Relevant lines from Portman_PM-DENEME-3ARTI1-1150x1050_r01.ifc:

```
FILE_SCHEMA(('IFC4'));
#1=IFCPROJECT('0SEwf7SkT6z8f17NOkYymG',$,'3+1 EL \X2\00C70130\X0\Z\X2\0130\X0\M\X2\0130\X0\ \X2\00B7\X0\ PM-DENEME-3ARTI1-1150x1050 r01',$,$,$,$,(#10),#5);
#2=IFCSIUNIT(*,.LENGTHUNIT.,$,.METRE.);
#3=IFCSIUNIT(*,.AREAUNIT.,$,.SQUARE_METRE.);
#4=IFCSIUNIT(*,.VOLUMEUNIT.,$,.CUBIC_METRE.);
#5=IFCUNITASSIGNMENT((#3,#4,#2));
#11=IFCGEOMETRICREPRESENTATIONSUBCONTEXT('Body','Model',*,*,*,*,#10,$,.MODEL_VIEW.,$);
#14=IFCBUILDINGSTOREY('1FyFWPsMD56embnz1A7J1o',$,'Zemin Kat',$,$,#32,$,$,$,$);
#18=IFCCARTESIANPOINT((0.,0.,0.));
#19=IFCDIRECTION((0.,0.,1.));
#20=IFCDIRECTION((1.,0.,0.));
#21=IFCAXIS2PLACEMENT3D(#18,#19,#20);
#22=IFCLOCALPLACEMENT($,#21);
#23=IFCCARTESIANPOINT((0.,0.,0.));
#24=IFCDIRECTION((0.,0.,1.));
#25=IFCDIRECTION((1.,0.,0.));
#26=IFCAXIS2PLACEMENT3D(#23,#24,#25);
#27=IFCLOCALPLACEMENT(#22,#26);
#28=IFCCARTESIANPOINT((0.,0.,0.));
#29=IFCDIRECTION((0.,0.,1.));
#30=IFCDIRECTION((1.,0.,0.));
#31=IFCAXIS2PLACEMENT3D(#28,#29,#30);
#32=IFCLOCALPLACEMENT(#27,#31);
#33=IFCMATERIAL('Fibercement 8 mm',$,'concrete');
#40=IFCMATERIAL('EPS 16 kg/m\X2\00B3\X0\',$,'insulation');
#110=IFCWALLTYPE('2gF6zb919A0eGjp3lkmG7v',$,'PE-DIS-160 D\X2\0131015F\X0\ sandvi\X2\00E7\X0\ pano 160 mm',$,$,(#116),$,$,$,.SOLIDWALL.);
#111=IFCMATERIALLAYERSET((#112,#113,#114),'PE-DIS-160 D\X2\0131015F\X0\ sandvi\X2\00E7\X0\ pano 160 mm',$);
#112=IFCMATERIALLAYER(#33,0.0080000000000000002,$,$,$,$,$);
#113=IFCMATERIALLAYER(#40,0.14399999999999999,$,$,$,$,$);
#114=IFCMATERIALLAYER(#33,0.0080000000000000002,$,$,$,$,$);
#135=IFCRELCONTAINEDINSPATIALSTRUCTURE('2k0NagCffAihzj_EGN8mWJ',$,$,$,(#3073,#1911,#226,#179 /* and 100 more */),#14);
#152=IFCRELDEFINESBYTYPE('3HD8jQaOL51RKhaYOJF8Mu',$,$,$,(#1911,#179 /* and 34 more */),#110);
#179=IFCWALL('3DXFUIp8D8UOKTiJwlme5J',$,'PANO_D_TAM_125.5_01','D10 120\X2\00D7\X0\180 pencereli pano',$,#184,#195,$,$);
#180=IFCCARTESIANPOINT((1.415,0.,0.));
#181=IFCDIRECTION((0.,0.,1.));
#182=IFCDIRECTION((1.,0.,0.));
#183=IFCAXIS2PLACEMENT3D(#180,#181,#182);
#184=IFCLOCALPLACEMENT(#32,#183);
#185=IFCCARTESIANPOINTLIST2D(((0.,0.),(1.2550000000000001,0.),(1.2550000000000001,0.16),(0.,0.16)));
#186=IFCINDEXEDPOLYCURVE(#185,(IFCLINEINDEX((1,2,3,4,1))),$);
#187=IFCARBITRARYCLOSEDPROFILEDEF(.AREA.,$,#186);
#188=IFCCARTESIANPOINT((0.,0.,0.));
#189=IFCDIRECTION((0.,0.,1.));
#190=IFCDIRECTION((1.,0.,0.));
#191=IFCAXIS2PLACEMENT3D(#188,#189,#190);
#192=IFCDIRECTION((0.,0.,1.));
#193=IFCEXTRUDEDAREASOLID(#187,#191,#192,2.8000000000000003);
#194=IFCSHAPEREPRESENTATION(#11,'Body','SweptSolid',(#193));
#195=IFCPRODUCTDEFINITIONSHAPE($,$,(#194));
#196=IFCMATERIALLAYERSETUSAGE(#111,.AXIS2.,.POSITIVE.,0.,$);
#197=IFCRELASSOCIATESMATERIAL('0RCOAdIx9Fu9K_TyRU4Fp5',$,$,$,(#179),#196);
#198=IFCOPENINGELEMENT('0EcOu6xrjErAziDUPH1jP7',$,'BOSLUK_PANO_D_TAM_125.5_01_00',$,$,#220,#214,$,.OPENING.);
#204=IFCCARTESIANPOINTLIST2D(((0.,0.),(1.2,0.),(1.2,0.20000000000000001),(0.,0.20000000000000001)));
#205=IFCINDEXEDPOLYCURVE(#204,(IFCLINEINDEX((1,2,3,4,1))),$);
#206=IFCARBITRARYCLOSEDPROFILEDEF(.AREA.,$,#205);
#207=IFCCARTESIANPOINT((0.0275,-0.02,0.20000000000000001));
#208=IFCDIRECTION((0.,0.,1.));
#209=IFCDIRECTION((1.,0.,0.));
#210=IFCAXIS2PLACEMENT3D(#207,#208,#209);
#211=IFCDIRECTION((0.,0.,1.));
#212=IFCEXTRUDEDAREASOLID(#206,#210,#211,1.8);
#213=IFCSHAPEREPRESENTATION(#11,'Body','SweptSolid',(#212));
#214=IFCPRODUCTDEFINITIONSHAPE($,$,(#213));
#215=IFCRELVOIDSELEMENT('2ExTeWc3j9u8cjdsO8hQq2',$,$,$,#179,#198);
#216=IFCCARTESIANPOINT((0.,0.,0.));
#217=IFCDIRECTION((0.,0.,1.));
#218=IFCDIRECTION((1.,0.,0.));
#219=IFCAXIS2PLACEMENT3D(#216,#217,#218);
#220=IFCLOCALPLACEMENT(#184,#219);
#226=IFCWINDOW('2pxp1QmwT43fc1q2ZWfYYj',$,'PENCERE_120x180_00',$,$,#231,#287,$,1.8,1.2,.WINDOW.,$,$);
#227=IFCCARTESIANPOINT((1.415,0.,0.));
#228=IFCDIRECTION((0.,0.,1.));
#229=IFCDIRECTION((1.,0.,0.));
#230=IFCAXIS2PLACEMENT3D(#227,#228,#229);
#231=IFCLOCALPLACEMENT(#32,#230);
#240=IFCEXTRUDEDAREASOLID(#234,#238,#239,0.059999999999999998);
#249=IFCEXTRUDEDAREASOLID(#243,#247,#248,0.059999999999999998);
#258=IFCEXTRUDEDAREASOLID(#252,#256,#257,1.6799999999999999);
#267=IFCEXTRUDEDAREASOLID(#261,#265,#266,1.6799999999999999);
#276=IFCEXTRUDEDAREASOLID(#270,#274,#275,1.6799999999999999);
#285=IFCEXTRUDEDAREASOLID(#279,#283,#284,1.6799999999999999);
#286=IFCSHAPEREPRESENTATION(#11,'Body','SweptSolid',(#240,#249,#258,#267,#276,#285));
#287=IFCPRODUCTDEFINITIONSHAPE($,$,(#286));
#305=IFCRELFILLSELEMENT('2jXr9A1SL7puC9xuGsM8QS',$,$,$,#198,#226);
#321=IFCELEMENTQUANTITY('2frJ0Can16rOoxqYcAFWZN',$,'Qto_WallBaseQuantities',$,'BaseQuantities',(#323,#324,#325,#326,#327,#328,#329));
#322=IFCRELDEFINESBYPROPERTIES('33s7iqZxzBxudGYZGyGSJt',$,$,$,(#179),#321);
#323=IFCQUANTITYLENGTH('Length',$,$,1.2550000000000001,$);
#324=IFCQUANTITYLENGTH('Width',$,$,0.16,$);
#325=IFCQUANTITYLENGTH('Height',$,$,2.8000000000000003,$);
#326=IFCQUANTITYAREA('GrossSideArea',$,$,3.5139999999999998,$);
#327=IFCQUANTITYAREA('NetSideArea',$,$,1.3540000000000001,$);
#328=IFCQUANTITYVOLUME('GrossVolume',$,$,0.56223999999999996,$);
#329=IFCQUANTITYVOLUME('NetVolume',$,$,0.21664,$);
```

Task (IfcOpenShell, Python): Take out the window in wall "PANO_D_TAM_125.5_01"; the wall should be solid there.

```python
import ifcopenshell
import ifcopenshell.api.feature
import ifcopenshell.api.pset
import ifcopenshell.api.root
import ifcopenshell.geom
import ifcopenshell.util.element
import ifcopenshell.util.shape
import ifcopenshell.util.unit

model = ifcopenshell.open("Portman_PM-DENEME-3ARTI1-1150x1050_r01.ifc")
area_scale = ifcopenshell.util.unit.calculate_unit_scale(model, "AREAUNIT")
volume_scale = ifcopenshell.util.unit.calculate_unit_scale(model, "VOLUMEUNIT")
settings = ifcopenshell.geom.settings()


def volume(element):
    """Net volume in cubic metres, openings subtracted."""
    shape = ifcopenshell.geom.create_shape(settings, element)
    return ifcopenshell.util.shape.get_volume(shape.geometry)


window = model.by_guid("2pxp1QmwT43fc1q2ZWfYYj")
opening = window.FillsVoids[0].RelatingOpeningElement
wall = opening.VoidsElements[0].RelatingBuildingElement
before = volume(wall)

ifcopenshell.api.root.remove_product(model, product=window)
ifcopenshell.api.feature.remove_feature(model, feature=opening)

after = volume(wall)
thickness = 0.16  # wall thickness in metres

# Update the wall's stored quantities.
qto = model.by_id(ifcopenshell.util.element.get_pset(wall, "Qto_WallBaseQuantities", should_inherit=False)["id"])
ifcopenshell.api.pset.edit_qto(model, qto=qto, properties={
    "NetSideArea": after / thickness / area_scale,
    "NetVolume": after / volume_scale,
})

print(f"wall volume {before:.3f} -> {after:.3f} m3")

model.write("Portman_PM-DENEME-3ARTI1-1150x1050_r01_rev.ifc")
```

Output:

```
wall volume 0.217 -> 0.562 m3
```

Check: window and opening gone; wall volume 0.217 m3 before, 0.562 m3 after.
